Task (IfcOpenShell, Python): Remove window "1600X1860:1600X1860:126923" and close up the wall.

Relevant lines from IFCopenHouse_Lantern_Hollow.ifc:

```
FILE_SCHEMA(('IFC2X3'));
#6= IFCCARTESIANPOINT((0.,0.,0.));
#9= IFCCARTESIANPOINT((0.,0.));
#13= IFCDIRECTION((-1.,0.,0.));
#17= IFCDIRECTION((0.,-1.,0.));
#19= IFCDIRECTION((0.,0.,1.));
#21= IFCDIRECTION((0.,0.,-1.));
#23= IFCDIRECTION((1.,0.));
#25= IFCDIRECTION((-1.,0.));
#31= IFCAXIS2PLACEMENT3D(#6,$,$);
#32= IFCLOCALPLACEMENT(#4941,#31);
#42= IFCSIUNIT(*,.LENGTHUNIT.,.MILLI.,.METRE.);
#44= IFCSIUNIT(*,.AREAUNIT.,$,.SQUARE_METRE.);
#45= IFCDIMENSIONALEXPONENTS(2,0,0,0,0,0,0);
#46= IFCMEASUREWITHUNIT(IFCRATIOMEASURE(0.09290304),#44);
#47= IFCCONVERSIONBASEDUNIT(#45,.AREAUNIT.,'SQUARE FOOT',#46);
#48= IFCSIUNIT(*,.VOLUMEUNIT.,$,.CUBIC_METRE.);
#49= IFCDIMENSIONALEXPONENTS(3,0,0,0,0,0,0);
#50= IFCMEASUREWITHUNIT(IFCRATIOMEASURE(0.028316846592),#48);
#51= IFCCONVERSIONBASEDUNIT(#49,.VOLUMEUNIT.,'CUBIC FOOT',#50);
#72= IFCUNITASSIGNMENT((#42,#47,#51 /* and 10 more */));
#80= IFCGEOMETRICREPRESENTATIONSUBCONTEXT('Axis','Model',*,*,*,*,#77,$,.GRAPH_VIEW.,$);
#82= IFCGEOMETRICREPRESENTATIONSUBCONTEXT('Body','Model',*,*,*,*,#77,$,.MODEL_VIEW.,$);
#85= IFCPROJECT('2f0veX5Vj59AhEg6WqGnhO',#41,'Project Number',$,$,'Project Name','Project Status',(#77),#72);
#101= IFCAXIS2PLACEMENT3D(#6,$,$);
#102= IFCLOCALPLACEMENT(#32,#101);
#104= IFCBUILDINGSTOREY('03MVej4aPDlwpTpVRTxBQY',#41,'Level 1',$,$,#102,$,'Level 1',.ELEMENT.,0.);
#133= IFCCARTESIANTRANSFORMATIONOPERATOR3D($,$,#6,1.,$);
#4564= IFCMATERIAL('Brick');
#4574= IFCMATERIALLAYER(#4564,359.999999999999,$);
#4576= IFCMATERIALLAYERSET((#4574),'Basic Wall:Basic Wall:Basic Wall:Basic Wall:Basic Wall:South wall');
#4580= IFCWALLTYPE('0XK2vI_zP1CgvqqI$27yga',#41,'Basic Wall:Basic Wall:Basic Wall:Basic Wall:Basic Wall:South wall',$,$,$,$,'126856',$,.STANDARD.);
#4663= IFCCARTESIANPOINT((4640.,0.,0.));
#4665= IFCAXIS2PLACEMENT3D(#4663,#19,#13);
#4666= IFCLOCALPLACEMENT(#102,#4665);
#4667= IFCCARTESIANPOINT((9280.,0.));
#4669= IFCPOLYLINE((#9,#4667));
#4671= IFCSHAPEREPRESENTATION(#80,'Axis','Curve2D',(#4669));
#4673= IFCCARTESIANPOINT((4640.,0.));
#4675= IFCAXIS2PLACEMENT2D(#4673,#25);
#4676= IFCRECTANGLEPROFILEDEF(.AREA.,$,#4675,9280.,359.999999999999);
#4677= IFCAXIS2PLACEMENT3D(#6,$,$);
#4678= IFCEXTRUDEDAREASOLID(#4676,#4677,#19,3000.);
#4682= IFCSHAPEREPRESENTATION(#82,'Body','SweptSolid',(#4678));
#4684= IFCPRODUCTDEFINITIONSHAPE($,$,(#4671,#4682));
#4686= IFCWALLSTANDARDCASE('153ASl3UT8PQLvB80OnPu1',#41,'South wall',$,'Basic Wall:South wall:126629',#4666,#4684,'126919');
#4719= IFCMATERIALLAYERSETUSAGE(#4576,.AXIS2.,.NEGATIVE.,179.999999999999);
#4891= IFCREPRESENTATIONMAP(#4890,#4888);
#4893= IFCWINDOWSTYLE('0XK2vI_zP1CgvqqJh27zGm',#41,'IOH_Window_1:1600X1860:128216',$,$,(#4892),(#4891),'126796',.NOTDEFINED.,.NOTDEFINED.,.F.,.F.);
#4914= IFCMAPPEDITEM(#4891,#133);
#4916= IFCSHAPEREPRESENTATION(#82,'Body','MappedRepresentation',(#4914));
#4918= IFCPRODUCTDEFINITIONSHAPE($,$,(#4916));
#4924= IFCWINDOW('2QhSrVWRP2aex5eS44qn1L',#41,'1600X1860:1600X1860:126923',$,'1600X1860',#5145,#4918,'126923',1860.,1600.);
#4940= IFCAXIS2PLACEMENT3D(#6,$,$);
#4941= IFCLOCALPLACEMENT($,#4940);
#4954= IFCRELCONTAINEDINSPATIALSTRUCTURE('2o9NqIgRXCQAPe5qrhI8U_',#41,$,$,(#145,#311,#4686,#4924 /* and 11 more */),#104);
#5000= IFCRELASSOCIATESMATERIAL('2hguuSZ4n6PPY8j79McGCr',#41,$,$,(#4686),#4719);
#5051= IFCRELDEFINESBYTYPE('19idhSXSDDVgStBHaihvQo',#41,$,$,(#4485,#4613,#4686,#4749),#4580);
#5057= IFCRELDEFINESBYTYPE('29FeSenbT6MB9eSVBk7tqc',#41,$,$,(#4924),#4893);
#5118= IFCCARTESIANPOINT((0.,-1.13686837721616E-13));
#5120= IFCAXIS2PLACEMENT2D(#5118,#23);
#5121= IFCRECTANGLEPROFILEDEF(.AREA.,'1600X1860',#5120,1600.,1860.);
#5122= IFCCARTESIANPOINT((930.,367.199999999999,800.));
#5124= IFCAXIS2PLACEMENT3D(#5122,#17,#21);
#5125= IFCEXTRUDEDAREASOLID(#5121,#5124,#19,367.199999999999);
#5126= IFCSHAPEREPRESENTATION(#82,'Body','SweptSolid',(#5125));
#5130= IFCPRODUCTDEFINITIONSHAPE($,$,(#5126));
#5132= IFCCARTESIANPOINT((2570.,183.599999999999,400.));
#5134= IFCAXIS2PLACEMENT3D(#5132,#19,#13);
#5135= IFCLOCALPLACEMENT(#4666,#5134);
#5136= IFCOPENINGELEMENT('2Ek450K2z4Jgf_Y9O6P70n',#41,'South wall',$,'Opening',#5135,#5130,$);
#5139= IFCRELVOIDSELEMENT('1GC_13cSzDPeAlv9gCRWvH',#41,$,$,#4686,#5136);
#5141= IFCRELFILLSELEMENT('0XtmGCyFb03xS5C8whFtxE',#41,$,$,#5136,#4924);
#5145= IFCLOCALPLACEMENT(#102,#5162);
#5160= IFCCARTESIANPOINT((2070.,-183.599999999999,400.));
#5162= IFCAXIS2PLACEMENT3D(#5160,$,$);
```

```python
import ifcopenshell
import ifcopenshell.api.feature
import ifcopenshell.api.root
import ifcopenshell.geom
import ifcopenshell.util.shape

model = ifcopenshell.open("IFCopenHouse_Lantern_Hollow.ifc")
settings = ifcopenshell.geom.settings()


def volume(element):
    """Net volume in cubic metres, openings subtracted."""
    shape = ifcopenshell.geom.create_shape(settings, element)
    return ifcopenshell.util.shape.get_volume(shape.geometry)


window = model.by_id(4924)
opening = window.FillsVoids[0].RelatingOpeningElement
wall = opening.VoidsElements[0].RelatingBuildingElement
before = volume(wall)

ifcopenshell.api.root.remove_product(model, product=window)
ifcopenshell.api.feature.remove_feature(model, feature=opening)

after = volume(wall)

print(f"wall volume {before:.3f} -> {after:.3f} m3")

model.write("IFCopenHouse_Lantern_Hollow_v2.ifc")
```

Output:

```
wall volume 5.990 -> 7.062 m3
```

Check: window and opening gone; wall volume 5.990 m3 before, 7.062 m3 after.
